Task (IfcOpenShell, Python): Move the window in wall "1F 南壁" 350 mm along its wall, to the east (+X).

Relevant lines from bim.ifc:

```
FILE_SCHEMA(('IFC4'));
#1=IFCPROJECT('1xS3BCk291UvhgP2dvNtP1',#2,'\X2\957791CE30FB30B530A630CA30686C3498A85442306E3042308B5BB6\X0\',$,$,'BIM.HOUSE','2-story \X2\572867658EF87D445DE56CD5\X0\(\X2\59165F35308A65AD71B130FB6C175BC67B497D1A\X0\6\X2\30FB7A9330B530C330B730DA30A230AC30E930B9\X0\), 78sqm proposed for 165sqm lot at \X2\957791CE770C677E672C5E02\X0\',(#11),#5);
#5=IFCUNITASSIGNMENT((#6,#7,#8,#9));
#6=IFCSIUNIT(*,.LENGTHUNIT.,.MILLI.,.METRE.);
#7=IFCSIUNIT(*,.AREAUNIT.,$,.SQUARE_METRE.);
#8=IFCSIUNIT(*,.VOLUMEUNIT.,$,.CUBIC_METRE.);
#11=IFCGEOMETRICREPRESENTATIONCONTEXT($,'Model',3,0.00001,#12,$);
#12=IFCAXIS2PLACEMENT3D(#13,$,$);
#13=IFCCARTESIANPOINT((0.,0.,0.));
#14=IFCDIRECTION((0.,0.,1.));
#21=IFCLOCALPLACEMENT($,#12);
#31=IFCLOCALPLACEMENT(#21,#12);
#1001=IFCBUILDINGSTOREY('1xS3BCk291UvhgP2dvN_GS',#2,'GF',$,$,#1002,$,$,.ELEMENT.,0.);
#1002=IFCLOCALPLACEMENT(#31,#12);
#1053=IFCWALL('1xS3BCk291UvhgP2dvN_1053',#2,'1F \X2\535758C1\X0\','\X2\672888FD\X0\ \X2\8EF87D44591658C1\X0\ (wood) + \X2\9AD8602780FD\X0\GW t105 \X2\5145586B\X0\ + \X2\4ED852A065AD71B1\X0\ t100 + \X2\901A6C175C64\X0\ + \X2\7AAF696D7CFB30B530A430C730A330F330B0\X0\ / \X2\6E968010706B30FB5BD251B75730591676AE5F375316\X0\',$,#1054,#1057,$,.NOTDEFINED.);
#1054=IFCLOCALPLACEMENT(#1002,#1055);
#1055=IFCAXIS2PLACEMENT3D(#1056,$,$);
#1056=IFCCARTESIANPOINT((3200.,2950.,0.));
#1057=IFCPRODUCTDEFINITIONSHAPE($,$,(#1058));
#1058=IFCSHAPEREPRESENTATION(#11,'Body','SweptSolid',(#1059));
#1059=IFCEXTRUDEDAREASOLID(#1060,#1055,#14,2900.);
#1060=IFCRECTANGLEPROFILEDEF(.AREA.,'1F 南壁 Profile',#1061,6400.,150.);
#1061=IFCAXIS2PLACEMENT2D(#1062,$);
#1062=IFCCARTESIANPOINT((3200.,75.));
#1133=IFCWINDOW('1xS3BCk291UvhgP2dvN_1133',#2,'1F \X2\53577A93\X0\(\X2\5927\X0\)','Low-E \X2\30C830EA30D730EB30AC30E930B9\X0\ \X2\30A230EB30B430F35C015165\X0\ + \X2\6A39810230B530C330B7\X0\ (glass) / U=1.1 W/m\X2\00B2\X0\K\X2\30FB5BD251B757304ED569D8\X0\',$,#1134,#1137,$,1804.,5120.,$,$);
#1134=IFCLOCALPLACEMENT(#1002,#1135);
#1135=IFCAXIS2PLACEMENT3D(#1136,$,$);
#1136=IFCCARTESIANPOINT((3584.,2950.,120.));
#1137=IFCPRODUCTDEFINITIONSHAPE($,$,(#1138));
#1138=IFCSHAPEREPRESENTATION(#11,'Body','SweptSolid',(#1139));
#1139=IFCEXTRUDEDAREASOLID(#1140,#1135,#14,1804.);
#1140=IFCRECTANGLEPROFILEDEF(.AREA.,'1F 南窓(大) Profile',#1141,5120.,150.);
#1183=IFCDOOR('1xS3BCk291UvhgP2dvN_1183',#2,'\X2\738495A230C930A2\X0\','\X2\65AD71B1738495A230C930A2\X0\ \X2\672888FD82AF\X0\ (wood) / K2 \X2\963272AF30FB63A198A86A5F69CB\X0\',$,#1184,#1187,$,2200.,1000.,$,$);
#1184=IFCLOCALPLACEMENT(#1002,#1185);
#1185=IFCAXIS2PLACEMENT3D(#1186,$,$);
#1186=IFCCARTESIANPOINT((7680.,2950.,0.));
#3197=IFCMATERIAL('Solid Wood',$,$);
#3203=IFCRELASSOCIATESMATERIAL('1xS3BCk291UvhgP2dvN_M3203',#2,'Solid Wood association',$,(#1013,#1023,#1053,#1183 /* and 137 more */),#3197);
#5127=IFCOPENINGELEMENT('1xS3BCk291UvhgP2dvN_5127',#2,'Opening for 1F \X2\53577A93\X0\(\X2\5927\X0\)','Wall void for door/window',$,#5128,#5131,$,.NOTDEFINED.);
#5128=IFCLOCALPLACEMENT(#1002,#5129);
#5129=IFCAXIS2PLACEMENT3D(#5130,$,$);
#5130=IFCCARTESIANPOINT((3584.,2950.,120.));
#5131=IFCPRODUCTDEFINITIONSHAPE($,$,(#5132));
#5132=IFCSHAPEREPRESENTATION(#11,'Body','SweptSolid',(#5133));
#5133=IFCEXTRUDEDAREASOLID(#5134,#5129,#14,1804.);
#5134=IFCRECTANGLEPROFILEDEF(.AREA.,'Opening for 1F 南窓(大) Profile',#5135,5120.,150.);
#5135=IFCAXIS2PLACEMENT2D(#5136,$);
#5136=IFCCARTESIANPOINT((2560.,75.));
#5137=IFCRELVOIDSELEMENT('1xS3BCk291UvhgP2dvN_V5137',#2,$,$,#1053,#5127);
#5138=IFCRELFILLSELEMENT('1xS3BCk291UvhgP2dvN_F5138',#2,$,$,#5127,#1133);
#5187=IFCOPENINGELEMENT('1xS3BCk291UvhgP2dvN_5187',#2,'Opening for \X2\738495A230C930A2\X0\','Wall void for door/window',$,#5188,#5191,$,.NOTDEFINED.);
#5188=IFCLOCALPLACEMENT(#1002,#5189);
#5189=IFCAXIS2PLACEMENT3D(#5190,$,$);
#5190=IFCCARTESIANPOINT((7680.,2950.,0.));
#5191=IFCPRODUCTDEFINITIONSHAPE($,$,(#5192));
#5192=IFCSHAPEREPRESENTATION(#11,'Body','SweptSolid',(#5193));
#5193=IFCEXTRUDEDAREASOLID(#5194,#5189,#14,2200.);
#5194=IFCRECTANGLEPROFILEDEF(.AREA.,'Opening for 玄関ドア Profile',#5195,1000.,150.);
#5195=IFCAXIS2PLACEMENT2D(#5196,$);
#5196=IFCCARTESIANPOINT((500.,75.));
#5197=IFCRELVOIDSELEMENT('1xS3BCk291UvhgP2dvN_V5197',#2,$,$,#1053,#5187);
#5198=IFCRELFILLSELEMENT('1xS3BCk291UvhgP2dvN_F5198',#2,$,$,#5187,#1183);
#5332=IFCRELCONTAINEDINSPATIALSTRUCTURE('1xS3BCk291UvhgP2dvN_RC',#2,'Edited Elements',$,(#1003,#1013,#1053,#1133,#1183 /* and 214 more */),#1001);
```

```python
import ifcopenshell
import ifcopenshell.api.geometry
import ifcopenshell.util.placement

model = ifcopenshell.open("bim.ifc")

window = model.by_id(1133)
opening = window.FillsVoids[0].RelatingOpeningElement
wall = opening.VoidsElements[0].RelatingBuildingElement

wall_matrix = ifcopenshell.util.placement.get_local_placement(wall.ObjectPlacement)
shift = wall_matrix[:3, 0] * 350.0
before = ifcopenshell.util.placement.get_local_placement(window.ObjectPlacement)[:3, 3].copy()

# The window is not placed relative to its opening, so move both.
for product in (opening, window):
    matrix = ifcopenshell.util.placement.get_local_placement(product.ObjectPlacement)
    matrix[:3, 3] += shift
    ifcopenshell.api.geometry.edit_object_placement(model, product=product, matrix=matrix, is_si=False)

after = ifcopenshell.util.placement.get_local_placement(window.ObjectPlacement)[:3, 3]
print("window moved by", (after - before).round(3) + 0.0)

model.write("bim-out.ifc")
```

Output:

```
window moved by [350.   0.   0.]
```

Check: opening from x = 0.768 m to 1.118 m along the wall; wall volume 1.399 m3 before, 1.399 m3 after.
